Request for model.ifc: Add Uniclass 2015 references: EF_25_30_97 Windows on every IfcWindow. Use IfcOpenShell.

First a look at what the model holds.

```python
import ifcopenshell

model = ifcopenshell.open("model.ifc")
print(model.schema)
print("classifications:", [c.Name for c in model.by_type("IfcClassification")])
for ifc_class in ("IfcDoor", "IfcRoof", "IfcStair", "IfcWall", "IfcWindow"):
    print(ifc_class, len(model.by_type(ifc_class)))
```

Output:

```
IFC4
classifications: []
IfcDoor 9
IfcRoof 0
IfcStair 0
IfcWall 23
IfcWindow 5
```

```python
import ifcopenshell
import ifcopenshell.api.classification

model = ifcopenshell.open("model.ifc")

system = ifcopenshell.api.classification.add_classification(model, classification="Uniclass 2015")

codes = {
    "IfcWindow": ("EF_25_30_97", "Windows"),
}
for ifc_class, (code, name) in codes.items():
    products = model.by_type(ifc_class)
    ifcopenshell.api.classification.add_reference(
        model, products=products, classification=system, identification=code, name=name
    )
    print(code, len(products))

model.write("model_updated.ifc")
```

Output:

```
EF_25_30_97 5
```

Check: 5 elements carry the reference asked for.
